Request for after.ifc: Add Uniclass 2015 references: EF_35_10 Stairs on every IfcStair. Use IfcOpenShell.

First a look at what the model holds.

```python
import ifcopenshell

model = ifcopenshell.open("after.ifc")
print(model.schema)
print("classifications:", [c.Name for c in model.by_type("IfcClassification")])
for ifc_class in ("IfcDoor", "IfcRoof", "IfcStair", "IfcWall", "IfcWindow"):
    print(ifc_class, len(model.by_type(ifc_class)))
```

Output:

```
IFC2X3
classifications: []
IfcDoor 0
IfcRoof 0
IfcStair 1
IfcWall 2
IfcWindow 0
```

```python
import ifcopenshell
import ifcopenshell.api.classification

model = ifcopenshell.open("after.ifc")

# IFC2X3 requires Source and Edition and has no link from the project to the system.
system = model.create_entity("IfcClassification", Source="NBS", Edition="2015", Name="Uniclass 2015")

codes = {
    "IfcStair": ("EF_35_10", "Stairs"),
}
for ifc_class, (code, name) in codes.items():
    products = model.by_type(ifc_class)
    ifcopenshell.api.classification.add_reference(
        model, products=products, classification=system, identification=code, name=name
    )
    print(code, len(products))

model.write("after_updated.ifc")
```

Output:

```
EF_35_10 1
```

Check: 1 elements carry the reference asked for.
